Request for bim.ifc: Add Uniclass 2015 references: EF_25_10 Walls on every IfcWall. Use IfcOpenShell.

First a look at what the model holds.

```python
import ifcopenshell

model = ifcopenshell.open("bim.ifc")
print(model.schema)
print("classifications:", [c.Name for c in model.by_type("IfcClassification")])
for ifc_class in ("IfcDoor", "IfcRoof", "IfcStair", "IfcWall", "IfcWindow"):
    print(ifc_class, len(model.by_type(ifc_class)))
```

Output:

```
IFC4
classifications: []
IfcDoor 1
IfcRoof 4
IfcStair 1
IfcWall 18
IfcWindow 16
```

```python
import ifcopenshell
import ifcopenshell.api.classification

model = ifcopenshell.open("bim.ifc")

system = ifcopenshell.api.classification.add_classification(model, classification="Uniclass 2015")

codes = {
    "IfcWall": ("EF_25_10", "Walls"),
}
for ifc_class, (code, name) in codes.items():
    products = model.by_type(ifc_class)
    ifcopenshell.api.classification.add_reference(
        model, products=products, classification=system, identification=code, name=name
    )
    print(code, len(products))

model.write("bim_updated.ifc")
```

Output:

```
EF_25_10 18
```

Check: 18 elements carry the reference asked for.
